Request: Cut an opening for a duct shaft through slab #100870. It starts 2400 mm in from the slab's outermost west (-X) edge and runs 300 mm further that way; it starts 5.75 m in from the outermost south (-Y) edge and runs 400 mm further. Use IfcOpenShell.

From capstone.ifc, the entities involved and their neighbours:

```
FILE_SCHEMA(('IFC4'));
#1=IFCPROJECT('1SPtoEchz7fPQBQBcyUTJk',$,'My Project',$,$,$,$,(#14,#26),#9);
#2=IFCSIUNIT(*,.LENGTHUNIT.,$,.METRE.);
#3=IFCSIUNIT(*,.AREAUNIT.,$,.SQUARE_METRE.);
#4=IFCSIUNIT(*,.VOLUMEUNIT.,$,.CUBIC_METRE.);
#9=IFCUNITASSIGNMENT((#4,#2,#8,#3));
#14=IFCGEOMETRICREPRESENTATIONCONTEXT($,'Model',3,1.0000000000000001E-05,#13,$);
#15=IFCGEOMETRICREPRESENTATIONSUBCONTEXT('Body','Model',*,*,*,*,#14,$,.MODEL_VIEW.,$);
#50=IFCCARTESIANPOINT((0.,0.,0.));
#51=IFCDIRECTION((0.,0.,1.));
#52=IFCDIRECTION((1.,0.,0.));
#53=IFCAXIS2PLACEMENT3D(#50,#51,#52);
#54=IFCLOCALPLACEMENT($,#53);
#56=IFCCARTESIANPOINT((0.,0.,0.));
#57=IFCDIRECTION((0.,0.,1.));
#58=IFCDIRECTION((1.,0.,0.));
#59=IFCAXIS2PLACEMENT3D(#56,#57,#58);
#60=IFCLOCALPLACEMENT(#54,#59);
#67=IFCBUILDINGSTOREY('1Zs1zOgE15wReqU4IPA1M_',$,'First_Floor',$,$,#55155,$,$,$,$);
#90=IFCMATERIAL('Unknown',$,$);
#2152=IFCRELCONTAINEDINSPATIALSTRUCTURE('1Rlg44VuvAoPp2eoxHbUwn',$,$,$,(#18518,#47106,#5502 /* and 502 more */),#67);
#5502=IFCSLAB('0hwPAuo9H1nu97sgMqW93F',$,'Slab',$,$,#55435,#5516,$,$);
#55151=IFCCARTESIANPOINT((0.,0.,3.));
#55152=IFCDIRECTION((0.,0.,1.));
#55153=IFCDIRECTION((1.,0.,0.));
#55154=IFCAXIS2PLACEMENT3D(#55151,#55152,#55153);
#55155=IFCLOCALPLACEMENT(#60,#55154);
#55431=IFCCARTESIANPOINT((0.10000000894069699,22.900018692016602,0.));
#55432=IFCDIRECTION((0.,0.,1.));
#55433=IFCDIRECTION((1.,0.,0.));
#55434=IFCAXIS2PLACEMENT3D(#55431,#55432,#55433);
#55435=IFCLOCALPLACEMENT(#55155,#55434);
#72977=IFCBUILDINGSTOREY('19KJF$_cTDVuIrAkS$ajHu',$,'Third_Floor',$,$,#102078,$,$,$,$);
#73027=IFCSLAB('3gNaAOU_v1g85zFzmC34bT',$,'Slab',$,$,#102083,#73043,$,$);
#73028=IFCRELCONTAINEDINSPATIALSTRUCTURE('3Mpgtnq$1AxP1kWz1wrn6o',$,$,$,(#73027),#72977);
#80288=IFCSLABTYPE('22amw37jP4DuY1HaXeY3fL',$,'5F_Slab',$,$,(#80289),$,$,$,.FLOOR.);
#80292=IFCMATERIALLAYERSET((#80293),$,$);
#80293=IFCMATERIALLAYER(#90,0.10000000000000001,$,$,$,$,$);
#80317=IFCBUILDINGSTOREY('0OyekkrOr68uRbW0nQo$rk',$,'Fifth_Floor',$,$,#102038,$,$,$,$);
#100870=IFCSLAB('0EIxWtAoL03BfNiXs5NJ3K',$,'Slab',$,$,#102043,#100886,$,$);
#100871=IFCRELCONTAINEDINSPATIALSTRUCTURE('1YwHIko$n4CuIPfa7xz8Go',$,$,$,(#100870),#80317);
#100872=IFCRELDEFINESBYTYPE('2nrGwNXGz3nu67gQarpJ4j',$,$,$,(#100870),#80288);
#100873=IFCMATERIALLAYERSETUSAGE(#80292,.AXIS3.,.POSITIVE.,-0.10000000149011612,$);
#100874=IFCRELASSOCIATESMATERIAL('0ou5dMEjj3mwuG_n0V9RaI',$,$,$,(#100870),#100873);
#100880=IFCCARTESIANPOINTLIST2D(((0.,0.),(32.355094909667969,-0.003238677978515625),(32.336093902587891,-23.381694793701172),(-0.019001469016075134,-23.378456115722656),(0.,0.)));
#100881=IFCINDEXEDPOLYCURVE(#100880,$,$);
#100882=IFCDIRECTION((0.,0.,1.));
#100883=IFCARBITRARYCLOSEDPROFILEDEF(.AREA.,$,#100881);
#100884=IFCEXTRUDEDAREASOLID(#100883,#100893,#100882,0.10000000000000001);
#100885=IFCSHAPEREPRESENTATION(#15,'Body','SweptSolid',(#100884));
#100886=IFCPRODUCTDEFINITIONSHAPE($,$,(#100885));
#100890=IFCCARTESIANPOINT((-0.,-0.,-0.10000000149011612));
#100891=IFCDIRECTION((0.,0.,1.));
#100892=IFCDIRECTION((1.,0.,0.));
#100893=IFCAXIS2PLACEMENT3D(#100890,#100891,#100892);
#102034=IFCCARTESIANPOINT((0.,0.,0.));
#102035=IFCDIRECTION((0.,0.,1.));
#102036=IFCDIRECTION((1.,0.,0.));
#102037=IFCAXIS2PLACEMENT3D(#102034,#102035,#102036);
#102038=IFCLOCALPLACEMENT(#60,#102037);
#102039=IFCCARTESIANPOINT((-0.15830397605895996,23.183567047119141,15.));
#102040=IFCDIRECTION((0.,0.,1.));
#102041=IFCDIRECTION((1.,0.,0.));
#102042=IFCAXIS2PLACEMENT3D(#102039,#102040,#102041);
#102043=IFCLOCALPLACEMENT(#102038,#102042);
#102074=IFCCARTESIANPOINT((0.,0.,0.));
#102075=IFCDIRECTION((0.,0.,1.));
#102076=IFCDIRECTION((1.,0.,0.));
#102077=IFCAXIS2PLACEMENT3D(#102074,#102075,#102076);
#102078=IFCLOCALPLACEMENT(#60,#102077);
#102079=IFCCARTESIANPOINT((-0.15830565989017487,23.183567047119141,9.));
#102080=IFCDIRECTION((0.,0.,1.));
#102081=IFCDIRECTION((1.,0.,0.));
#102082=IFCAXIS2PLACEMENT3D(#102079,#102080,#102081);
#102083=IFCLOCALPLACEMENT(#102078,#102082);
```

```python
import numpy as np
import ifcopenshell
import ifcopenshell.api.feature
import ifcopenshell.api.geometry
import ifcopenshell.api.root
import ifcopenshell.geom
import ifcopenshell.util.placement
import ifcopenshell.util.representation
import ifcopenshell.util.shape
import ifcopenshell.util.unit

model = ifcopenshell.open("capstone.ifc")
unit_scale = ifcopenshell.util.unit.calculate_unit_scale(model)
settings = ifcopenshell.geom.settings()


def volume(element):
    """Net volume in cubic metres, openings subtracted."""
    shape = ifcopenshell.geom.create_shape(settings, element)
    return ifcopenshell.util.shape.get_volume(shape.geometry)


slab = model.by_id(100870)
before = volume(slab)

# Extent in the slab's own axes, in metres. The edges named are its -X and -Y sides.
slab_shape = ifcopenshell.geom.create_shape(settings, slab)
vertices = ifcopenshell.util.shape.get_vertices(slab_shape.geometry)
x_min, y_min, bottom = vertices.min(axis=0)
top = vertices[:, 2].max()

opening = ifcopenshell.api.root.create_entity(model, ifc_class="IfcOpeningElement", name="Duct shaft opening", predefined_type="OPENING")
context = ifcopenshell.util.representation.get_context(model, "Model", "Body", "MODEL_VIEW")
width, depth = 0.3, 0.4
outline = [(0.0, 0.0), (width, 0.0), (width, depth), (0.0, depth), (0.0, 0.0)]
# Overshoot both faces by 50 mm so the cut is clean.
shape = ifcopenshell.api.geometry.add_slab_representation(
    model, context=context, depth=top - bottom + 0.1, polyline=outline
)
ifcopenshell.api.geometry.assign_representation(model, product=opening, representation=shape)

matrix = ifcopenshell.util.placement.get_local_placement(slab.ObjectPlacement)
matrix[:, 3] = matrix @ np.append(np.array([x_min + 2.4, y_min + 5.75, bottom - 0.05]) / unit_scale, 1.0)
ifcopenshell.api.geometry.edit_object_placement(model, product=opening, matrix=matrix, is_si=False)
ifcopenshell.api.feature.add_feature(model, feature=opening, element=slab)

after = volume(slab)

print(f"slab volume {before:.3f} -> {after:.3f} m3")

model.write("capstone_rev.ifc")
```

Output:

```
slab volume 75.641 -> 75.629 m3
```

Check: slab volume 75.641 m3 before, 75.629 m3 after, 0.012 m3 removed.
